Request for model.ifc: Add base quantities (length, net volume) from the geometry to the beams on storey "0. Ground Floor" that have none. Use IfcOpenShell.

First a look at what the model holds.

```python
import ifcopenshell
import ifcopenshell.util.element
import ifcopenshell.util.unit

model = ifcopenshell.open("model.ifc")
print(model.schema)
for unit_type in ("LENGTHUNIT", "AREAUNIT", "VOLUMEUNIT"):
    print(unit_type, ifcopenshell.util.unit.calculate_unit_scale(model, unit_type))
storey = next(s for s in model.by_type("IfcBuildingStorey") if s.Name == "0. Ground Floor")
beams = [e for e in ifcopenshell.util.element.get_decomposition(storey) if e.is_a("IfcBeam")]
for e in sorted(beams, key=lambda e: e.id()):
    print(e.id(), e.is_a(), e.Name, list(ifcopenshell.util.element.get_psets(e, qtos_only=True)), sep=" | ")
```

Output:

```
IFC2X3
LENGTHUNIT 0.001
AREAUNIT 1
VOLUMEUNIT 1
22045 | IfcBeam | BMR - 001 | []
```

```python
import ifcopenshell
import ifcopenshell.api.pset
import ifcopenshell.geom
import ifcopenshell.util.element
import ifcopenshell.util.shape
import ifcopenshell.util.unit

model = ifcopenshell.open("model.ifc")
unit_scale = ifcopenshell.util.unit.calculate_unit_scale(model)
volume_scale = ifcopenshell.util.unit.calculate_unit_scale(model, "VOLUMEUNIT")
settings = ifcopenshell.geom.settings()

storey = next(s for s in model.by_type("IfcBuildingStorey") if s.Name == "0. Ground Floor")
beams = [e for e in ifcopenshell.util.element.get_decomposition(storey) if e.is_a("IfcBeam")]

for e in sorted(beams, key=lambda e: e.id()):
    if ifcopenshell.util.element.get_psets(e, qtos_only=True, should_inherit=False):
        continue
    # Geometry comes back in metres, in the element's own axes.
    shape = ifcopenshell.geom.create_shape(settings, e)
    values = {
        "Length": ifcopenshell.util.shape.get_max_xyz(shape.geometry) / unit_scale,
        "NetVolume": ifcopenshell.util.shape.get_volume(shape.geometry) / volume_scale,
    }
    qto = ifcopenshell.api.pset.add_qto(model, product=e, name="BaseQuantities")
    ifcopenshell.api.pset.edit_qto(model, qto=qto, properties=values)
    print(e.id(), {k: round(v, 3) for k, v in values.items()})

model.write("model_v2.ifc")
```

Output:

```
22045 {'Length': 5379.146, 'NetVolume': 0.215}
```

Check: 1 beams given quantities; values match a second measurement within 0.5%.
